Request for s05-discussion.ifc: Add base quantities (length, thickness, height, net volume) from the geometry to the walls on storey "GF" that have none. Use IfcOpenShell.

First a look at what the model holds.

```python
import ifcopenshell
import ifcopenshell.util.element
import ifcopenshell.util.unit

model = ifcopenshell.open("s05-discussion.ifc")
print(model.schema)
for unit_type in ("LENGTHUNIT", "AREAUNIT", "VOLUMEUNIT"):
    print(unit_type, ifcopenshell.util.unit.calculate_unit_scale(model, unit_type))
storey = next(s for s in model.by_type("IfcBuildingStorey") if s.Name == "GF")
walls = [e for e in ifcopenshell.util.element.get_decomposition(storey) if e.is_a("IfcWall")]
for e in sorted(walls, key=lambda e: e.id()):
    print(e.id(), e.is_a(), e.Name, list(ifcopenshell.util.element.get_psets(e, qtos_only=True)), sep=" | ")
```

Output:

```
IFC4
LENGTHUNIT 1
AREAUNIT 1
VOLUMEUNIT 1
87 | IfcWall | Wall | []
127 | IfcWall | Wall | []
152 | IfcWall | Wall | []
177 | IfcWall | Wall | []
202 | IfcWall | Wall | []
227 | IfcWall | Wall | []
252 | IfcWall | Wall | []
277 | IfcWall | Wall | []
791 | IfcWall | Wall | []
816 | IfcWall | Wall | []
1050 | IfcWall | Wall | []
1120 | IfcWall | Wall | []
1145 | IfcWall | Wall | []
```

```python
import ifcopenshell
import ifcopenshell.api.pset
import ifcopenshell.geom
import ifcopenshell.util.element
import ifcopenshell.util.shape
import ifcopenshell.util.unit

model = ifcopenshell.open("s05-discussion.ifc")
unit_scale = ifcopenshell.util.unit.calculate_unit_scale(model)
volume_scale = ifcopenshell.util.unit.calculate_unit_scale(model, "VOLUMEUNIT")
settings = ifcopenshell.geom.settings()

storey = next(s for s in model.by_type("IfcBuildingStorey") if s.Name == "GF")
walls = [e for e in ifcopenshell.util.element.get_decomposition(storey) if e.is_a("IfcWall")]

for e in sorted(walls, key=lambda e: e.id()):
    if ifcopenshell.util.element.get_psets(e, qtos_only=True, should_inherit=False):
        continue
    # Geometry comes back in metres, in the element's own axes.
    shape = ifcopenshell.geom.create_shape(settings, e)
    values = {
        "Length": ifcopenshell.util.shape.get_x(shape.geometry) / unit_scale,
        "Width": ifcopenshell.util.shape.get_y(shape.geometry) / unit_scale,
        "Height": ifcopenshell.util.shape.get_z(shape.geometry) / unit_scale,
        "NetVolume": ifcopenshell.util.shape.get_volume(shape.geometry) / volume_scale,
    }
    qto = ifcopenshell.api.pset.add_qto(model, product=e, name="Qto_WallBaseQuantities")
    ifcopenshell.api.pset.edit_qto(model, qto=qto, properties=values)
    print(e.id(), {k: round(v, 3) for k, v in values.items()})

model.write("s05-discussion_updated.ifc")
```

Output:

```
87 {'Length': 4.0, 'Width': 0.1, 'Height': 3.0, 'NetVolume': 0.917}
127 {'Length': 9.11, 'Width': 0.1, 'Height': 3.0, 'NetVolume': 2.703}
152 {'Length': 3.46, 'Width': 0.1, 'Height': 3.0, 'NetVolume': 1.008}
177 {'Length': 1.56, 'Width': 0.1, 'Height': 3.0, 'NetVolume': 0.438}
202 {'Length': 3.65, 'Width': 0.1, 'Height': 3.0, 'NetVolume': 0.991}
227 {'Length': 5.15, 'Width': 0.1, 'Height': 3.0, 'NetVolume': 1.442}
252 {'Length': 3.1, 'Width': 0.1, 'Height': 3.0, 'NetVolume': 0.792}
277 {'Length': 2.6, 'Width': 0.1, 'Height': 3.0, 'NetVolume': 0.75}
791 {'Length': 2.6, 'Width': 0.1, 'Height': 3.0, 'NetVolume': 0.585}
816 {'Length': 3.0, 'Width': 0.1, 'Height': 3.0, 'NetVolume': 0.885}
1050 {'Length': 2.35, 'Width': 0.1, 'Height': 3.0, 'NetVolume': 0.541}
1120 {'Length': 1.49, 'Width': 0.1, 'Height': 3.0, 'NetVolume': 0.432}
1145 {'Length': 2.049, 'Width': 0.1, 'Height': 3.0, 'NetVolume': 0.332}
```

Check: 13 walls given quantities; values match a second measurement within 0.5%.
